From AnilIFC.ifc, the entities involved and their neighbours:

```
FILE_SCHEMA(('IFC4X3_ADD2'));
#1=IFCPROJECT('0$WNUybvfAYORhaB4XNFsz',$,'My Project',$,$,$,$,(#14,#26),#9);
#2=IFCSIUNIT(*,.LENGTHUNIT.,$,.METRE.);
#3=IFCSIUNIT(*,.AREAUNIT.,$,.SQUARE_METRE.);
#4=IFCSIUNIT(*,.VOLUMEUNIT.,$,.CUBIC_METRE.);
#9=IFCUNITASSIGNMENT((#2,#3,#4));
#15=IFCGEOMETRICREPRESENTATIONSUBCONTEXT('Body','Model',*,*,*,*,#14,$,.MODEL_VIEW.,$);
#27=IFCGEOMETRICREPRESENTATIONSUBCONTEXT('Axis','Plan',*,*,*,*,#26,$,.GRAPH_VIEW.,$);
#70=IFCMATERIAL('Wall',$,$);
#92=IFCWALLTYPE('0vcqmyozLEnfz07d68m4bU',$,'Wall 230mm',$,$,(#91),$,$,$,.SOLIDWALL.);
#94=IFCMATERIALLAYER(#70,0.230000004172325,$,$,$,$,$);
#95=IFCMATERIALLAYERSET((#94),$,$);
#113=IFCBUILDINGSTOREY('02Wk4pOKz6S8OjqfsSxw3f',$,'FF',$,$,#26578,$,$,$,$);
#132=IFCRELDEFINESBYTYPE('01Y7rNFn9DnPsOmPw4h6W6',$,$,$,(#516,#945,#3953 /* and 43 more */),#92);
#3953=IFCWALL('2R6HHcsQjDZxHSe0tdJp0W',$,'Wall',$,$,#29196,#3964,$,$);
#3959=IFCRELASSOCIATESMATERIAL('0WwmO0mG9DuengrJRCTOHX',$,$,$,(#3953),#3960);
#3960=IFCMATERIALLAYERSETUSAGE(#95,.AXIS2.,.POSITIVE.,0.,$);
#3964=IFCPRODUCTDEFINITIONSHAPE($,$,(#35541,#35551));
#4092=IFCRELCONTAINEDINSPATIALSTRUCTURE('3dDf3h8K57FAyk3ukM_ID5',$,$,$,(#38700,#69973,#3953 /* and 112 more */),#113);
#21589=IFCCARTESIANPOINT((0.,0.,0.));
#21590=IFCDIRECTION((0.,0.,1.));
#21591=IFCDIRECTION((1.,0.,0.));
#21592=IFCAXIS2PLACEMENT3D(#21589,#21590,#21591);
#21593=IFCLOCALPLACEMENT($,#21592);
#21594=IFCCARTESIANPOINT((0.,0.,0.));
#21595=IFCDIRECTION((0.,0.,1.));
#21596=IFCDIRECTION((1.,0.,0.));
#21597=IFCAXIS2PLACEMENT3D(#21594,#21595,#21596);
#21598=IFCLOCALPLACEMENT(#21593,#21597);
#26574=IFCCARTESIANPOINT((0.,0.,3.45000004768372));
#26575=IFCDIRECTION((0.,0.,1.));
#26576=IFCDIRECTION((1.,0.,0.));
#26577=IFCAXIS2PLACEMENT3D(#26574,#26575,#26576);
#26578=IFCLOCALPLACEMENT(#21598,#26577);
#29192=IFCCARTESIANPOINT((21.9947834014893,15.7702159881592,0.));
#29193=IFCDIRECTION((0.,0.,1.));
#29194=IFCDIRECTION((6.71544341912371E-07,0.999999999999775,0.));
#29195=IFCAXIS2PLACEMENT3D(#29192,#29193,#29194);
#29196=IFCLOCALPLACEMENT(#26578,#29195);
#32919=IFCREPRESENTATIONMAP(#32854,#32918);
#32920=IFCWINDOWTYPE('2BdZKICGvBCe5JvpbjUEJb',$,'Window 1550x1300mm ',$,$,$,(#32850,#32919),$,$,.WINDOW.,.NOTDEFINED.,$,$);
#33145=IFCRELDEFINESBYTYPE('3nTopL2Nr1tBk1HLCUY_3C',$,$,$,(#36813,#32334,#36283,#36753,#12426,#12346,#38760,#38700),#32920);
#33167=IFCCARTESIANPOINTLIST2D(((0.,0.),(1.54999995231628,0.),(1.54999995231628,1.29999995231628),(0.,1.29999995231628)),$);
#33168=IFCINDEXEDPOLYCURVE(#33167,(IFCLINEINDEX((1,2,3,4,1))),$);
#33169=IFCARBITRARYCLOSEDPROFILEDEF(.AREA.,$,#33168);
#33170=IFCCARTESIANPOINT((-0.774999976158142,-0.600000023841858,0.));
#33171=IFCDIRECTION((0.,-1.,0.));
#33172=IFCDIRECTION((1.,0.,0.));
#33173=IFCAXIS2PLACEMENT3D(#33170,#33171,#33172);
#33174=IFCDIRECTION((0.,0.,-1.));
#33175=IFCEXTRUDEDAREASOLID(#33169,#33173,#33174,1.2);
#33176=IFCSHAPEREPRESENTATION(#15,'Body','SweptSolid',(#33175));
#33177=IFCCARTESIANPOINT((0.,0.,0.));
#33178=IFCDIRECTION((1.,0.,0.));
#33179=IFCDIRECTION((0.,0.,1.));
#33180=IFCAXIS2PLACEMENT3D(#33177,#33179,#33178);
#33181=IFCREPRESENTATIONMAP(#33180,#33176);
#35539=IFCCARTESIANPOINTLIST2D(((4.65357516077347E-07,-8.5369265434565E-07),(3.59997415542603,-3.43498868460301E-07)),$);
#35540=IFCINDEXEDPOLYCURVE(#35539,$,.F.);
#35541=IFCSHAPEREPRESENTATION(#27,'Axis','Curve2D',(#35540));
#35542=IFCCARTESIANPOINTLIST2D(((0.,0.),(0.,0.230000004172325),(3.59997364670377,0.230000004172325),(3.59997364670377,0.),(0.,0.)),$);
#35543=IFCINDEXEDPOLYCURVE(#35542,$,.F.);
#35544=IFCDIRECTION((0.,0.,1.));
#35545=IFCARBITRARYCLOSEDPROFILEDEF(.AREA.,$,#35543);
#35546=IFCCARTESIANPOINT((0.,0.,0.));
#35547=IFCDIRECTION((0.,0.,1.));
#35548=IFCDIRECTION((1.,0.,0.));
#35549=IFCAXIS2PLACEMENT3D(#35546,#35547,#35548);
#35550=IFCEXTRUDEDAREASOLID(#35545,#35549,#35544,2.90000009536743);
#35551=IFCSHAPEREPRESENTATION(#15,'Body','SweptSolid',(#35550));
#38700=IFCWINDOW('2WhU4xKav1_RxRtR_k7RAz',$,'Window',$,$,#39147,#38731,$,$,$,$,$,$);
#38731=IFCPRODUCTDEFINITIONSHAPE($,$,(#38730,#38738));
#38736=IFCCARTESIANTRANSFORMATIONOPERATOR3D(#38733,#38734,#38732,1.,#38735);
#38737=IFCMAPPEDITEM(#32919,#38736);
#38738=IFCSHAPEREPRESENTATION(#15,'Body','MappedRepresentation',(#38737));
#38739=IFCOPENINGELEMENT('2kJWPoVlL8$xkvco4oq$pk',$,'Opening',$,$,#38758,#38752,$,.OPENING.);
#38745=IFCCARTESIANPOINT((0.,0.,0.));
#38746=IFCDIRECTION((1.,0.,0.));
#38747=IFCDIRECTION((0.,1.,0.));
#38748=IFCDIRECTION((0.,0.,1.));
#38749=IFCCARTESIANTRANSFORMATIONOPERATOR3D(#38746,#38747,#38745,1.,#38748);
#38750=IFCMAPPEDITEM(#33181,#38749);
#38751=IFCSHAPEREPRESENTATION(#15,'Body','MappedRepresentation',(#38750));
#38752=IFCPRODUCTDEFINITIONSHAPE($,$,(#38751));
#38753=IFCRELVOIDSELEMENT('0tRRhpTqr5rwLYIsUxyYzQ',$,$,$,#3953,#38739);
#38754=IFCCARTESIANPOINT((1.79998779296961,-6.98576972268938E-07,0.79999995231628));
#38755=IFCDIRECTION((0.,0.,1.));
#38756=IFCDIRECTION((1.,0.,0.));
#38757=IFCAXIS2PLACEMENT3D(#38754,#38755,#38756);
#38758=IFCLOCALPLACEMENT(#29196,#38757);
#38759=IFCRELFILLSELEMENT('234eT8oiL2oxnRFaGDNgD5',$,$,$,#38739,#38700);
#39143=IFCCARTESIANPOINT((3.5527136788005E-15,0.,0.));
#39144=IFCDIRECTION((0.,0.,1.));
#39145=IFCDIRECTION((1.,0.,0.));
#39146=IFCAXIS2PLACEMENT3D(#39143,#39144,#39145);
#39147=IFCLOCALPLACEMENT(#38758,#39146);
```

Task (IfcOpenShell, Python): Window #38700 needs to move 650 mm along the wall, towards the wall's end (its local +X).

```python
import ifcopenshell
import ifcopenshell.api.geometry
import ifcopenshell.util.placement
import ifcopenshell.util.unit

model = ifcopenshell.open("AnilIFC.ifc")
unit_scale = ifcopenshell.util.unit.calculate_unit_scale(model)

window = model.by_guid("2WhU4xKav1_RxRtR_k7RAz")
opening = window.FillsVoids[0].RelatingOpeningElement
wall = opening.VoidsElements[0].RelatingBuildingElement

wall_matrix = ifcopenshell.util.placement.get_local_placement(wall.ObjectPlacement)
shift = wall_matrix[:3, 0] * 0.65 / unit_scale
before = ifcopenshell.util.placement.get_local_placement(window.ObjectPlacement)[:3, 3].copy()

# The window is placed relative to its opening, so it follows when the opening moves.
matrix = ifcopenshell.util.placement.get_local_placement(opening.ObjectPlacement)
matrix[:3, 3] += shift
ifcopenshell.api.geometry.edit_object_placement(
    model, product=opening, matrix=matrix, is_si=False, should_transform_children=True
)

after = ifcopenshell.util.placement.get_local_placement(window.ObjectPlacement)[:3, 3]
print("window moved by", (after - before).round(3) + 0.0)

model.write("AnilIFC-out.ifc")
```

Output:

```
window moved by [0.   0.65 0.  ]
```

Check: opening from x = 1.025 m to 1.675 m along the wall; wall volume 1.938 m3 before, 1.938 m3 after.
